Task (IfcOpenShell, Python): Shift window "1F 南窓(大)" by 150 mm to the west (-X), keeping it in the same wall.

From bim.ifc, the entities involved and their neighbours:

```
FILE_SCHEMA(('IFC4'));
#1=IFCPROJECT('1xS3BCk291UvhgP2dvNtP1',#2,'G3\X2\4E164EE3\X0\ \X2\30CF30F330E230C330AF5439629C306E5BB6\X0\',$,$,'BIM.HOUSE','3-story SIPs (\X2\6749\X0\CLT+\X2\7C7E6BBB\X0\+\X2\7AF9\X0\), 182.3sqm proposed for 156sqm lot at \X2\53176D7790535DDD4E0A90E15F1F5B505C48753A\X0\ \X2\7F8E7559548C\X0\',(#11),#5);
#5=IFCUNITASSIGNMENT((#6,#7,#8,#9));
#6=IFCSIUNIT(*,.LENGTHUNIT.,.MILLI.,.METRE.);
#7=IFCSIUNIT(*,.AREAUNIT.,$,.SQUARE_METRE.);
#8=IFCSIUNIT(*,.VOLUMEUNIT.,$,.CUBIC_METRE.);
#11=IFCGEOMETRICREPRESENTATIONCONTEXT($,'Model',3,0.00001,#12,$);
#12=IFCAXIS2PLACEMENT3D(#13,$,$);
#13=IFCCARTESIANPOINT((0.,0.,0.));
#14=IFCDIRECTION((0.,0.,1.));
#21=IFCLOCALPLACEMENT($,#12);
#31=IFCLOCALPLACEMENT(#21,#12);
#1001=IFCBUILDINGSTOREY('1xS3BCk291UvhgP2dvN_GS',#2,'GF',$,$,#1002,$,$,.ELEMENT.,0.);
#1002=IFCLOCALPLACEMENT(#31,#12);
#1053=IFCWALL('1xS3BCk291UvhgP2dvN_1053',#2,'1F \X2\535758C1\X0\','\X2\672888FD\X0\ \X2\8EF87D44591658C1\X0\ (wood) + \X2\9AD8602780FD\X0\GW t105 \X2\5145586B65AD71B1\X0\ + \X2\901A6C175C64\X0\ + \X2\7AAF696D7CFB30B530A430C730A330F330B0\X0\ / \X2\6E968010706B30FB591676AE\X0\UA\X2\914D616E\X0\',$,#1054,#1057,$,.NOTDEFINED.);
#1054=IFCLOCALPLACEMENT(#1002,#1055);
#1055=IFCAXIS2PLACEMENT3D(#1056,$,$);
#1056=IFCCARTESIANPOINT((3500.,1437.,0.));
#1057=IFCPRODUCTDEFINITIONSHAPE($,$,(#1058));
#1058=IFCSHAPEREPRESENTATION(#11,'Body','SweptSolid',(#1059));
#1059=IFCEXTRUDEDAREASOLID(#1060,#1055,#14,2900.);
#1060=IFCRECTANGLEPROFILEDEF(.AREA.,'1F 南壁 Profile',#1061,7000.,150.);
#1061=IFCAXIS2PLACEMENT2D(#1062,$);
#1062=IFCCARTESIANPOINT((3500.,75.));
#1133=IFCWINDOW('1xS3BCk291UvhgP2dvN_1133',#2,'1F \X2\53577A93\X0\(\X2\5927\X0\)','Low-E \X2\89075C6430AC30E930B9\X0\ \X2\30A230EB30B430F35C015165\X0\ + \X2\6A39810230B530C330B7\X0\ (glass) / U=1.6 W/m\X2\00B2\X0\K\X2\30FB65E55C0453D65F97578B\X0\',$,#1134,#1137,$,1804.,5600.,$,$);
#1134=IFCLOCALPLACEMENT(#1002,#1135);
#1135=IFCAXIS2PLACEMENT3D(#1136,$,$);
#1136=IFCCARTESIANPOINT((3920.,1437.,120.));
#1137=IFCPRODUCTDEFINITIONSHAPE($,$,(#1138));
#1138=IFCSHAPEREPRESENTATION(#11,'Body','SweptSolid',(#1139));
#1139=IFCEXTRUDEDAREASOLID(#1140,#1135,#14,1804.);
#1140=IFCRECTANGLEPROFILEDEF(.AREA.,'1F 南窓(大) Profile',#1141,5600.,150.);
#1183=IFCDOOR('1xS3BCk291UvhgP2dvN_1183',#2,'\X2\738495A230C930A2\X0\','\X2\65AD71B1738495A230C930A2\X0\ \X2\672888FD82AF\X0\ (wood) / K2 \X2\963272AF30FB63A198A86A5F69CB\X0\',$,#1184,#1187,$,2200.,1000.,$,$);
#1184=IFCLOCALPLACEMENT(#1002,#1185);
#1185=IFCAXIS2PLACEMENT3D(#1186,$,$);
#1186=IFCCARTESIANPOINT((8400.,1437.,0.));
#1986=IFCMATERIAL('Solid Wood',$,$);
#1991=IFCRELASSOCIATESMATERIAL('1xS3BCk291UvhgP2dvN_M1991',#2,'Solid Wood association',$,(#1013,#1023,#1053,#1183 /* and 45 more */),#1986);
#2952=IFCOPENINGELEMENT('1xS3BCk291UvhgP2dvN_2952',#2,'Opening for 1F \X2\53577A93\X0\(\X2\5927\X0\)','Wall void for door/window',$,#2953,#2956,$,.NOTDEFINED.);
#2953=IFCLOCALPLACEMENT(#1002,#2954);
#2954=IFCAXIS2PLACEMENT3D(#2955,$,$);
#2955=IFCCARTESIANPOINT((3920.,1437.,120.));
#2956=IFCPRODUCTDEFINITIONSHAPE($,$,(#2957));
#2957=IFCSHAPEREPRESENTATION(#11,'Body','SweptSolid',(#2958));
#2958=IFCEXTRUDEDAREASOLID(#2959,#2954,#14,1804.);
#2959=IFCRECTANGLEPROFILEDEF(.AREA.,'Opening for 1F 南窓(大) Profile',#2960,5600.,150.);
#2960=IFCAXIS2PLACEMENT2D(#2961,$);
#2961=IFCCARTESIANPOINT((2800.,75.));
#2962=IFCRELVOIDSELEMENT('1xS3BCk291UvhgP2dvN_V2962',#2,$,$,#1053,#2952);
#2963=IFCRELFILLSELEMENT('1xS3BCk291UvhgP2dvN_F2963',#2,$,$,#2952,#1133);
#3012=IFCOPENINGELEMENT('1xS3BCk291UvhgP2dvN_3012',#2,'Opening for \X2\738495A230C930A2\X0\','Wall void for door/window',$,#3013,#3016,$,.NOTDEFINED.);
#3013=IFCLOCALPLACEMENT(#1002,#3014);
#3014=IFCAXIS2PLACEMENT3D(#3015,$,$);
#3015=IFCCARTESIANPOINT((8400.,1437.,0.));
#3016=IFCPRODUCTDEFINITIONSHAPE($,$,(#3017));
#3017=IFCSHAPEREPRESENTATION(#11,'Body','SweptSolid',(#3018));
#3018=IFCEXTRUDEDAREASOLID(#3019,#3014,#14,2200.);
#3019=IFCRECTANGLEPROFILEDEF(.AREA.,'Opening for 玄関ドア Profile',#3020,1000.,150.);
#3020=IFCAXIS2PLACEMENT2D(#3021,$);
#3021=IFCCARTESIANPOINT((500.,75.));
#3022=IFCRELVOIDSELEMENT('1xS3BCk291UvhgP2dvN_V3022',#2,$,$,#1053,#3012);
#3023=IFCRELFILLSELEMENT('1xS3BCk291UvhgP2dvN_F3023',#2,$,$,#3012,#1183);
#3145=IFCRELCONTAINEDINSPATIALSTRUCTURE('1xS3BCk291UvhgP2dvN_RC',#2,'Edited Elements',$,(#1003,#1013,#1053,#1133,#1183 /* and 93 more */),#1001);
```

```python
import ifcopenshell
import ifcopenshell.api.geometry
import ifcopenshell.util.placement
import ifcopenshell.util.unit

model = ifcopenshell.open("bim.ifc")
unit_scale = ifcopenshell.util.unit.calculate_unit_scale(model)

window = model.by_guid("1xS3BCk291UvhgP2dvN_1133")
opening = window.FillsVoids[0].RelatingOpeningElement
wall = opening.VoidsElements[0].RelatingBuildingElement

wall_matrix = ifcopenshell.util.placement.get_local_placement(wall.ObjectPlacement)
shift = wall_matrix[:3, 0] * -0.15 / unit_scale
before = ifcopenshell.util.placement.get_local_placement(window.ObjectPlacement)[:3, 3].copy()

# The window is not placed relative to its opening, so move both.
for product in (opening, window):
    matrix = ifcopenshell.util.placement.get_local_placement(product.ObjectPlacement)
    matrix[:3, 3] += shift
    ifcopenshell.api.geometry.edit_object_placement(model, product=product, matrix=matrix, is_si=False)

after = ifcopenshell.util.placement.get_local_placement(window.ObjectPlacement)[:3, 3]
print("window moved by", (after - before).round(3) + 0.0)

model.write("bim_rev.ifc")
```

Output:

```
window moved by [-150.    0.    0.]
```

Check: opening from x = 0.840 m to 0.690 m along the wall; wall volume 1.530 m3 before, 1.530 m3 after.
